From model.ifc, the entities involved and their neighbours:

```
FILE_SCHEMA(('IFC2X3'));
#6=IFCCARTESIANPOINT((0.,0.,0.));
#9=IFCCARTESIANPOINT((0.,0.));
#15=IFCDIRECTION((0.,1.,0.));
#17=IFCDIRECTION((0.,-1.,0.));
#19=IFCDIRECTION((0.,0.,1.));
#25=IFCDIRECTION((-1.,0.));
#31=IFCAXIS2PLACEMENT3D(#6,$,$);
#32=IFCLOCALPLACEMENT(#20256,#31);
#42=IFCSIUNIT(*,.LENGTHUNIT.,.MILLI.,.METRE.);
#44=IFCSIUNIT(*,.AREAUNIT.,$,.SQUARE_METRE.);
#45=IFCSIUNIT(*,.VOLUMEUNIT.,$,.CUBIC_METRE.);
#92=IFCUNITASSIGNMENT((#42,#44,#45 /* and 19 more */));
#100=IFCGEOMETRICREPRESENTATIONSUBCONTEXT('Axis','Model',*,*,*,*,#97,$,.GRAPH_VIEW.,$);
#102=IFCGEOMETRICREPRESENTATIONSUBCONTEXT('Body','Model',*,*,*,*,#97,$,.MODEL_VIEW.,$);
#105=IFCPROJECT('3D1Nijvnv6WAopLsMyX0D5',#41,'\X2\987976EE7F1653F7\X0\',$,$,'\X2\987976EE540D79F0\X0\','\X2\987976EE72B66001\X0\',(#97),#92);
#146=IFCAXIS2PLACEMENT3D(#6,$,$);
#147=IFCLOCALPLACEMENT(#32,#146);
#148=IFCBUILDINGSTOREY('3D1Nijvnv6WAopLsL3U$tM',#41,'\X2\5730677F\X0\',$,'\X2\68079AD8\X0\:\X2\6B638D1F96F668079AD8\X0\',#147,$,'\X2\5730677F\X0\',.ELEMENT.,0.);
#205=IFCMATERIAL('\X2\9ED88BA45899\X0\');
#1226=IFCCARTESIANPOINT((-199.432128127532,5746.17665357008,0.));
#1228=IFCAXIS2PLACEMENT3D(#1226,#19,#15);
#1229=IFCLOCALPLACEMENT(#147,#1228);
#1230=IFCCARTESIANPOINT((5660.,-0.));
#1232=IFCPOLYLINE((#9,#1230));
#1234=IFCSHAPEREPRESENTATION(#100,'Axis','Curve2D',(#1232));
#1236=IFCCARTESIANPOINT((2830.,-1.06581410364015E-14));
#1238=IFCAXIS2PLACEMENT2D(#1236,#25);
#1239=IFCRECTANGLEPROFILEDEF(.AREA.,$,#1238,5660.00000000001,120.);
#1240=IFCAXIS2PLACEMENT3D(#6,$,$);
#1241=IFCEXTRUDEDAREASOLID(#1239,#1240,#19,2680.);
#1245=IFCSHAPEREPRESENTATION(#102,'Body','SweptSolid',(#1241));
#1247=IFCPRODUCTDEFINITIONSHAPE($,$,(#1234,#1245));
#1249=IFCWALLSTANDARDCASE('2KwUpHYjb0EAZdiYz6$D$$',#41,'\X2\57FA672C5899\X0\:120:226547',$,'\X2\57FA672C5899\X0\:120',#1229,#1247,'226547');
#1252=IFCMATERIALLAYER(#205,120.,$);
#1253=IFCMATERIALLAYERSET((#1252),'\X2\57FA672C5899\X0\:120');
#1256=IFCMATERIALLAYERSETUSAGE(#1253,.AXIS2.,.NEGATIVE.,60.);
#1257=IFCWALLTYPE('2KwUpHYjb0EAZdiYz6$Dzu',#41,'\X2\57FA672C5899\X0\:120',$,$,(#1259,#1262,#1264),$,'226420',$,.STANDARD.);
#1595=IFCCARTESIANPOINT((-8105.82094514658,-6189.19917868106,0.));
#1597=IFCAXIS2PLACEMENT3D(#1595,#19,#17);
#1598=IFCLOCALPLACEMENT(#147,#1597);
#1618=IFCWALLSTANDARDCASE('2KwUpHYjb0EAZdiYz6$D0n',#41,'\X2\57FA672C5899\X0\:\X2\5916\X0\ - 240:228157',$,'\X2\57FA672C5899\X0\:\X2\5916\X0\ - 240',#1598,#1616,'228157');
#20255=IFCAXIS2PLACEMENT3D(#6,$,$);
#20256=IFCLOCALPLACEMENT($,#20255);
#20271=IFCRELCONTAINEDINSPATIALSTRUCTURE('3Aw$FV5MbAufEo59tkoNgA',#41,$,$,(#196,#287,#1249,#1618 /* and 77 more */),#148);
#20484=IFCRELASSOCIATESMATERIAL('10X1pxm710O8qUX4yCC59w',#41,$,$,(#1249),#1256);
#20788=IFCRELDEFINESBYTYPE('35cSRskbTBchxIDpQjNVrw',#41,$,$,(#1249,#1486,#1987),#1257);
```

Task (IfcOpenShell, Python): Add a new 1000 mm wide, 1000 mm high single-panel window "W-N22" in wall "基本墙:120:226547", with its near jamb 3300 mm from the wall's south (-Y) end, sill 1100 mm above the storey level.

```python
import numpy as np
import ifcopenshell
import ifcopenshell.api.feature
import ifcopenshell.api.geometry
import ifcopenshell.api.root
import ifcopenshell.api.spatial
import ifcopenshell.api.type
import ifcopenshell.geom
import ifcopenshell.util.element
import ifcopenshell.util.placement
import ifcopenshell.util.representation
import ifcopenshell.util.shape
import ifcopenshell.util.unit

model = ifcopenshell.open("model.ifc")
unit_scale = ifcopenshell.util.unit.calculate_unit_scale(model)
settings = ifcopenshell.geom.settings()


def volume(element):
    """Net volume in cubic metres, openings subtracted."""
    shape = ifcopenshell.geom.create_shape(settings, element)
    return ifcopenshell.util.shape.get_volume(shape.geometry)


wall = model.by_id(1249)
storey = ifcopenshell.util.element.get_container(wall, ifc_class="IfcBuildingStorey")
context = ifcopenshell.util.representation.get_context(model, "Model", "Body", "MODEL_VIEW")
before = volume(wall)

width, height, from_end, sill = 1, 1, 3.3, 1.1  # metres

# The wall runs along its own X axis, and the end named is its -X end.
wall_shape = ifcopenshell.geom.create_shape(settings, wall)
x, y, z = ifcopenshell.util.shape.get_vertices(wall_shape.geometry).T
start = x.min() + from_end
face, thickness = float(y.min()), float(y.max() - y.min())
wall_matrix = ifcopenshell.util.placement.get_local_placement(wall.ObjectPlacement)
level = ifcopenshell.util.placement.get_local_placement(storey.ObjectPlacement)[2, 3]


def in_wall(x, y):
    """Placement at x, y metres in the wall's axes, at sill height."""
    matrix = wall_matrix.copy()
    matrix[:, 3] = wall_matrix @ np.array([x / unit_scale, y / unit_scale, 0.0, 1.0])
    matrix[2, 3] = level + sill / unit_scale
    return matrix


# Opening: a box that overshoots both wall faces by 50 mm.
opening = ifcopenshell.api.root.create_entity(model, ifc_class="IfcOpeningElement")
box = ifcopenshell.api.geometry.add_wall_representation(
    model, context=context, length=width, height=height, thickness=thickness + 0.1
)
ifcopenshell.api.geometry.assign_representation(model, product=opening, representation=box)
ifcopenshell.api.geometry.edit_object_placement(model, product=opening, matrix=in_wall(start, face - 0.05), is_si=False)
ifcopenshell.api.feature.add_feature(model, feature=opening, element=wall)

window = ifcopenshell.api.root.create_entity(model, ifc_class="IfcWindow", name="W-N22")
window.OverallWidth, window.OverallHeight = width / unit_scale, height / unit_scale
body = ifcopenshell.api.geometry.add_window_representation(
    model,
    context=context,
    overall_width=window.OverallWidth,
    overall_height=window.OverallHeight,
    partition_type="SINGLE_PANEL",
)
ifcopenshell.api.geometry.assign_representation(model, product=window, representation=body)
ifcopenshell.api.spatial.assign_container(model, products=[window], relating_structure=storey)
fills = ifcopenshell.api.feature.add_filling(model, opening=opening, element=window)
fills.OwnerHistory = window.OwnerHistory  # required in IFC2X3

# IFC2X3 keeps the operation on the window style.
style = ifcopenshell.api.root.create_entity(model, ifc_class="IfcWindowStyle", name="W-N22")
style.OperationType, style.ConstructionType = "SINGLE_PANEL", "NOTDEFINED"
style.ParameterTakesPrecedence = style.Sizeable = False
ifcopenshell.api.type.assign_type(model, related_objects=[window], relating_type=style)

# Centre the window in the wall's thickness.
ifcopenshell.api.geometry.edit_object_placement(model, product=window, matrix=in_wall(start, face), is_si=False)
window_shape = ifcopenshell.geom.create_shape(settings, window)
depth = ifcopenshell.util.shape.get_vertices(window_shape.geometry)[:, 1]
offset = face + thickness / 2 - (depth.min() + depth.max()) / 2
ifcopenshell.api.geometry.edit_object_placement(model, product=window, matrix=in_wall(start, offset), is_si=False)

after = volume(wall)

print(f"wall volume {before:.3f} -> {after:.3f} m3")

model.write("model_edited.ifc")
```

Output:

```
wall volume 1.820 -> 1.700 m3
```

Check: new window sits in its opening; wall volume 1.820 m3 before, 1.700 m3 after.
